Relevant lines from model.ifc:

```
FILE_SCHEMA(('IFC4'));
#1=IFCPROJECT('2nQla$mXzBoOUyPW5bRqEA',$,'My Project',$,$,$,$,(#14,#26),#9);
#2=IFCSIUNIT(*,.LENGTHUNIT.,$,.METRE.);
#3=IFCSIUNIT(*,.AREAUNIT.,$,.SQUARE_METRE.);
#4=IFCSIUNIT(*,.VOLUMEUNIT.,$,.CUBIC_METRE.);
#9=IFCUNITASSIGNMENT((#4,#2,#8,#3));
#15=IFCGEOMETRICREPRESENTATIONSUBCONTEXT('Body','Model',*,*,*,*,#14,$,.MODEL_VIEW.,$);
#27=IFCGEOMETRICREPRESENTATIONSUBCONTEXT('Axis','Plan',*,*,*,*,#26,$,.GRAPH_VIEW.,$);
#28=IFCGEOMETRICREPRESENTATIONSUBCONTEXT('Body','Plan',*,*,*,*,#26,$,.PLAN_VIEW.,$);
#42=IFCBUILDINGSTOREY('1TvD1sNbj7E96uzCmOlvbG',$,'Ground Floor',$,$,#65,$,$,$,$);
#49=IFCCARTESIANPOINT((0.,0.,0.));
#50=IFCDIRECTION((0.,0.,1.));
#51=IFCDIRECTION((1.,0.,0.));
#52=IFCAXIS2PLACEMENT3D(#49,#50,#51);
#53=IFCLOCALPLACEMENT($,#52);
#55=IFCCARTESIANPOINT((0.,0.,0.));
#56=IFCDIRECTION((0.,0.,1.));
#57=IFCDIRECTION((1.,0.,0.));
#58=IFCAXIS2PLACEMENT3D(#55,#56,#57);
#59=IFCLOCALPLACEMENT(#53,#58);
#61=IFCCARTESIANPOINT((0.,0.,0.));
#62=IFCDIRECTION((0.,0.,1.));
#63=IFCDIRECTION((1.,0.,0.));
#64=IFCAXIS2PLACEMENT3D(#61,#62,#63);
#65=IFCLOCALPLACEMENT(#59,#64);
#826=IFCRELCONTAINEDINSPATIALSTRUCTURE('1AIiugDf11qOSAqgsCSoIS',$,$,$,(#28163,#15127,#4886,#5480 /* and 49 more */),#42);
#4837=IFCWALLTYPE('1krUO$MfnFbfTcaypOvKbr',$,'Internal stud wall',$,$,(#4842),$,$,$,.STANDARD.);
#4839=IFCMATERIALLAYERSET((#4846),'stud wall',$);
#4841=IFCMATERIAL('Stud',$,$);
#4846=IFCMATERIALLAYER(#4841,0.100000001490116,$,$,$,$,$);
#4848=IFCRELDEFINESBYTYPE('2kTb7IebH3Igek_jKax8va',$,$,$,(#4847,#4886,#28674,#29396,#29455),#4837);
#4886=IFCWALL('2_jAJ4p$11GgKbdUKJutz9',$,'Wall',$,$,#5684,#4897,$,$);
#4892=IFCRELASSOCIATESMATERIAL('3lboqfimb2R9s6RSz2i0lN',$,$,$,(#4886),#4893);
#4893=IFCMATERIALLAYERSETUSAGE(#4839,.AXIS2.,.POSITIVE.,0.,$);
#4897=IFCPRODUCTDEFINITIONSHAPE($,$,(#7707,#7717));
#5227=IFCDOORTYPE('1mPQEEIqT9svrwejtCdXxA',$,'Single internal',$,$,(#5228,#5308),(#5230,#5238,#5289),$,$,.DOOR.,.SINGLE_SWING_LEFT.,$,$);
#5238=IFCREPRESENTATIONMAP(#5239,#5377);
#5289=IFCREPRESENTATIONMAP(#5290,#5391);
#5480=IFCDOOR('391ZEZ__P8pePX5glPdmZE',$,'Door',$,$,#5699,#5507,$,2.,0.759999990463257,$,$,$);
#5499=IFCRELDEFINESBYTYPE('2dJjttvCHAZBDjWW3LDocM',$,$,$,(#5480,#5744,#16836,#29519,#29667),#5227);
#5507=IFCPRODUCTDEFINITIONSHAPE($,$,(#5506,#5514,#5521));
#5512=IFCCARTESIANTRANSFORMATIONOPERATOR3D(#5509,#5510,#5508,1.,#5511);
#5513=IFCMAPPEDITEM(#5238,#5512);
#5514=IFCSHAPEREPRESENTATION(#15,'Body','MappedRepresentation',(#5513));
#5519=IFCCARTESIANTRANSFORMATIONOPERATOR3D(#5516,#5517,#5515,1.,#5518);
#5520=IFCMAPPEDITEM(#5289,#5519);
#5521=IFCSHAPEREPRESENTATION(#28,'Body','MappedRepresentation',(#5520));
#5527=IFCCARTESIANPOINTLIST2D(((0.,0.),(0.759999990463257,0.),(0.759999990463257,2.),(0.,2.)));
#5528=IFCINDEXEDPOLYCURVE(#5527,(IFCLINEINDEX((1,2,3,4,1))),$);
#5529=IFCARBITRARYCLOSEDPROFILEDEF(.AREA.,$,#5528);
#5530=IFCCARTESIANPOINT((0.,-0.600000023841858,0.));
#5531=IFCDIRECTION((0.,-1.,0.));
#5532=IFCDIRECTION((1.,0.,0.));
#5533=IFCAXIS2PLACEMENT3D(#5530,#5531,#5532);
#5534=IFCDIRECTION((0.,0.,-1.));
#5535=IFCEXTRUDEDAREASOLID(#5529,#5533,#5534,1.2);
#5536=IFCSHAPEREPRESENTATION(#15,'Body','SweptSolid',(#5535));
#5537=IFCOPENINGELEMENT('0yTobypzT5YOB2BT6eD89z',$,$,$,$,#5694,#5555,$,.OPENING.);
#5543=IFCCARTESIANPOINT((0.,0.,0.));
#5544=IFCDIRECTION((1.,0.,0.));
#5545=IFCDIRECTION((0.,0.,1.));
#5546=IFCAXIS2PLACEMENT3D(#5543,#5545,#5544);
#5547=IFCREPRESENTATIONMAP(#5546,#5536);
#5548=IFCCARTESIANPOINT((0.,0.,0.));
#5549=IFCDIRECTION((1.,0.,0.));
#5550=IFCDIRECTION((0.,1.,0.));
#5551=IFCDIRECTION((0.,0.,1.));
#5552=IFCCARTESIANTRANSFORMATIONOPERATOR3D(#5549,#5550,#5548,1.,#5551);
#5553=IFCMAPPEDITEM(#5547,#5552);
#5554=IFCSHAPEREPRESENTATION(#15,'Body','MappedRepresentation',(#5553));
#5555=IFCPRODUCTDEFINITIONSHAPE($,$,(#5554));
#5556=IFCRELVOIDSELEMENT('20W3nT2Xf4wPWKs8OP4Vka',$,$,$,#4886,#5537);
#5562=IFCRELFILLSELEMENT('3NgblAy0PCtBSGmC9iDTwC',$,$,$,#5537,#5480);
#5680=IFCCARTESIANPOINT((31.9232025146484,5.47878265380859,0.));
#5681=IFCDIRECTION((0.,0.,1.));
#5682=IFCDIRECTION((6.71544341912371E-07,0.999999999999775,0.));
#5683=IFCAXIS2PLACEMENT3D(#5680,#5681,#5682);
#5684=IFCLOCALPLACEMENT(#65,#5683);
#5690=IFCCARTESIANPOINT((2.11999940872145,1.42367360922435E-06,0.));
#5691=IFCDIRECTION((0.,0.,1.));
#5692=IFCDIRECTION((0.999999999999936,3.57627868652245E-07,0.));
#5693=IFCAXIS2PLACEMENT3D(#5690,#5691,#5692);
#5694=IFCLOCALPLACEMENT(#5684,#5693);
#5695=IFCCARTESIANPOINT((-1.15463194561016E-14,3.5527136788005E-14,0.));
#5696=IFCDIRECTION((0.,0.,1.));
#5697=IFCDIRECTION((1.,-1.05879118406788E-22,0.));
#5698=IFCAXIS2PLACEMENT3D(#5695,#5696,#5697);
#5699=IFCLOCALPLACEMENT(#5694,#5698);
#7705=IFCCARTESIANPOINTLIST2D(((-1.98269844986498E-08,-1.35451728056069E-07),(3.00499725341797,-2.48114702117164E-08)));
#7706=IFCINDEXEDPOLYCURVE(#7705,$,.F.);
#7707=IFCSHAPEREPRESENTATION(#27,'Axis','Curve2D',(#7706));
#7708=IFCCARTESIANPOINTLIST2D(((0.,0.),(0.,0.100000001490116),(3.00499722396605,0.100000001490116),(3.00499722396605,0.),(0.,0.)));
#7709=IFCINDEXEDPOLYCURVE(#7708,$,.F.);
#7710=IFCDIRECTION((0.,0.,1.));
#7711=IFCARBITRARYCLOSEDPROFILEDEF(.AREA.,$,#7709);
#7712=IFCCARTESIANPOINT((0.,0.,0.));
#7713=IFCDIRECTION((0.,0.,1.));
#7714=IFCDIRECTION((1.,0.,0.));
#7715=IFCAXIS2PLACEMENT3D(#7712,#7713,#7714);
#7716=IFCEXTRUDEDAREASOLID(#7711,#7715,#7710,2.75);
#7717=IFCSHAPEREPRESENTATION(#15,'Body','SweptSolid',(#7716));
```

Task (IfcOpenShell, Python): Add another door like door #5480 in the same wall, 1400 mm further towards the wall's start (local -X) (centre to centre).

```python
import ifcopenshell
import ifcopenshell.api.feature
import ifcopenshell.api.geometry
import ifcopenshell.api.root
import ifcopenshell.geom
import ifcopenshell.util.element
import ifcopenshell.util.placement
import ifcopenshell.util.shape
import ifcopenshell.util.unit

model = ifcopenshell.open("model.ifc")
unit_scale = ifcopenshell.util.unit.calculate_unit_scale(model)
settings = ifcopenshell.geom.settings()


def volume(element):
    """Net volume in cubic metres, openings subtracted."""
    shape = ifcopenshell.geom.create_shape(settings, element)
    return ifcopenshell.util.shape.get_volume(shape.geometry)


door = model.by_guid("391ZEZ__P8pePX5glPdmZE")
opening = door.FillsVoids[0].RelatingOpeningElement
wall = opening.VoidsElements[0].RelatingBuildingElement
before = volume(wall)
shift = ifcopenshell.util.placement.get_local_placement(wall.ObjectPlacement)[:3, 0] * -1.4 / unit_scale

# copy_class copies the void relationship, type, container and properties, but no geometry.
new_opening = ifcopenshell.api.root.copy_class(model, product=opening)
new_opening.Representation = ifcopenshell.util.element.copy_deep(
    model, opening.Representation, exclude=["IfcGeometricRepresentationContext", "IfcRepresentationMap"]
)
new_door = ifcopenshell.api.root.copy_class(model, product=door)
new_door.Representation = ifcopenshell.util.element.copy_deep(
    model, door.Representation, exclude=["IfcGeometricRepresentationContext", "IfcRepresentationMap"]
)
ifcopenshell.api.feature.add_filling(model, opening=new_opening, element=new_door)

for old, new in ((opening, new_opening), (door, new_door)):
    matrix = ifcopenshell.util.placement.get_local_placement(old.ObjectPlacement)
    matrix[:3, 3] += shift
    ifcopenshell.api.geometry.edit_object_placement(model, product=new, matrix=matrix, is_si=False)

after = volume(wall)

print(f"wall volume {before:.3f} -> {after:.3f} m3")

model.write("model_updated.ifc")
```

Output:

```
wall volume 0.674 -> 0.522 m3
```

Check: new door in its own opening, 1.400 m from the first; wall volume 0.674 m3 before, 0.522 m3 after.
